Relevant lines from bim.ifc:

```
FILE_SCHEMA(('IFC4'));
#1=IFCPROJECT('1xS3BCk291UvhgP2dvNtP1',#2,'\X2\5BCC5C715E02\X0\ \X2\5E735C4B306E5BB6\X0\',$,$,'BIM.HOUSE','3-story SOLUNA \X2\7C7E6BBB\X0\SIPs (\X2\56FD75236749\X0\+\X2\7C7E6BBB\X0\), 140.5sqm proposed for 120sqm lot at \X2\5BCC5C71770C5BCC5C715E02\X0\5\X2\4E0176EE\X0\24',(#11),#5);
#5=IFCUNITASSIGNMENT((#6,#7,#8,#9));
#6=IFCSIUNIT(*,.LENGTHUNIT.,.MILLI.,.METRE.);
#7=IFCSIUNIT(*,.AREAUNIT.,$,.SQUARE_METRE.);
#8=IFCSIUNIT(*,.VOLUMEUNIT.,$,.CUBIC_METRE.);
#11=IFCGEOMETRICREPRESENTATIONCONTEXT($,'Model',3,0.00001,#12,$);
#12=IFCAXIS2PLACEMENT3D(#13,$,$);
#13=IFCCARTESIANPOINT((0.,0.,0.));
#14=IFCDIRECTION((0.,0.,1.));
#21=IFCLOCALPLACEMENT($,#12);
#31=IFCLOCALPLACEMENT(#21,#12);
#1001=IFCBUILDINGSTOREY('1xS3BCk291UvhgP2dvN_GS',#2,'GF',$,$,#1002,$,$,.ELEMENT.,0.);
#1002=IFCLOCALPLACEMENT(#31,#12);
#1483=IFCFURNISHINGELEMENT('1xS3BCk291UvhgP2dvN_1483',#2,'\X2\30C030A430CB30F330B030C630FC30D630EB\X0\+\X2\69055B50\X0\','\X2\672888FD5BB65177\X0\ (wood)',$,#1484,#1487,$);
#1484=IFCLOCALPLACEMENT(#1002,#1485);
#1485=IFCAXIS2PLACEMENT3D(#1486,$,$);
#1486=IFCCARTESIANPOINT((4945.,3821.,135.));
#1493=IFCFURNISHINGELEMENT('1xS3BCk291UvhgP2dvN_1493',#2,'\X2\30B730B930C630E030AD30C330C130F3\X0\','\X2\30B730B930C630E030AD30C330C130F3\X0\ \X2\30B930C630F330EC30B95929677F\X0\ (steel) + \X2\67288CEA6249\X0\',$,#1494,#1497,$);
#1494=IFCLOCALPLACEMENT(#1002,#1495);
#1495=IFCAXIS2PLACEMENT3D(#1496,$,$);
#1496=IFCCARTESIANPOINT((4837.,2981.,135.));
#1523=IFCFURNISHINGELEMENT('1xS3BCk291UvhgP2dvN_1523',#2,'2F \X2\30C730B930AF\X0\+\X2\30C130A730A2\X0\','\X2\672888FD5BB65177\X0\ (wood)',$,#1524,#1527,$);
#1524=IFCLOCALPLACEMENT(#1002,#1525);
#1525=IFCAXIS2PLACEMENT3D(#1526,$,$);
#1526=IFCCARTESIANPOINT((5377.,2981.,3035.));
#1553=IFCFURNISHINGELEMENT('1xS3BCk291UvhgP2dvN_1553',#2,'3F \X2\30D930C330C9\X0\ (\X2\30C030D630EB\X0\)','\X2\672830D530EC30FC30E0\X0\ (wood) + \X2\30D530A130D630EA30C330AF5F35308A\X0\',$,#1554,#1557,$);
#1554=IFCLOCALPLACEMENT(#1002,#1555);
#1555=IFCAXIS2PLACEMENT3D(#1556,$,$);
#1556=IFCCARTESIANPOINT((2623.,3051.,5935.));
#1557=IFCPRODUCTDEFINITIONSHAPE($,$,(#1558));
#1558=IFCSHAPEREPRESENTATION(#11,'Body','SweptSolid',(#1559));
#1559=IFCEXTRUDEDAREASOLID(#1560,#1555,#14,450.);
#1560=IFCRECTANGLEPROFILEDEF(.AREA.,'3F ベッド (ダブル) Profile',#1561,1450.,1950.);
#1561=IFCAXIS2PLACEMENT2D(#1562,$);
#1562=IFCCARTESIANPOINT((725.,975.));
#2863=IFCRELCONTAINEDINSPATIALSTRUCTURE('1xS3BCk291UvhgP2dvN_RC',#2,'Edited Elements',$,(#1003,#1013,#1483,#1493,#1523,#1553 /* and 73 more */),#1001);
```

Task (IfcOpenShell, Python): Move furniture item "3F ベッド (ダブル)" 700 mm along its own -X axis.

```python
import ifcopenshell
import ifcopenshell.api.geometry
import ifcopenshell.util.placement
import ifcopenshell.util.unit

model = ifcopenshell.open("bim.ifc")
unit_scale = ifcopenshell.util.unit.calculate_unit_scale(model)

item = model.by_guid("1xS3BCk291UvhgP2dvN_1553")
matrix = ifcopenshell.util.placement.get_local_placement(item.ObjectPlacement)
matrix[:3, 3] -= matrix[:3, 0] * 0.7 / unit_scale
ifcopenshell.api.geometry.edit_object_placement(model, product=item, matrix=matrix, is_si=False)

print(ifcopenshell.util.placement.get_local_placement(item.ObjectPlacement).round(3) + 0.0)

model.write("bim-out.ifc")
```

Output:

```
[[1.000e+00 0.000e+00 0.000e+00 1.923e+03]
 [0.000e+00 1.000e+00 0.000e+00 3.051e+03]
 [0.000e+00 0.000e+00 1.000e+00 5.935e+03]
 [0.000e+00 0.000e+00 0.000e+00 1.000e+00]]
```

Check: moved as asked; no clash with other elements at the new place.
